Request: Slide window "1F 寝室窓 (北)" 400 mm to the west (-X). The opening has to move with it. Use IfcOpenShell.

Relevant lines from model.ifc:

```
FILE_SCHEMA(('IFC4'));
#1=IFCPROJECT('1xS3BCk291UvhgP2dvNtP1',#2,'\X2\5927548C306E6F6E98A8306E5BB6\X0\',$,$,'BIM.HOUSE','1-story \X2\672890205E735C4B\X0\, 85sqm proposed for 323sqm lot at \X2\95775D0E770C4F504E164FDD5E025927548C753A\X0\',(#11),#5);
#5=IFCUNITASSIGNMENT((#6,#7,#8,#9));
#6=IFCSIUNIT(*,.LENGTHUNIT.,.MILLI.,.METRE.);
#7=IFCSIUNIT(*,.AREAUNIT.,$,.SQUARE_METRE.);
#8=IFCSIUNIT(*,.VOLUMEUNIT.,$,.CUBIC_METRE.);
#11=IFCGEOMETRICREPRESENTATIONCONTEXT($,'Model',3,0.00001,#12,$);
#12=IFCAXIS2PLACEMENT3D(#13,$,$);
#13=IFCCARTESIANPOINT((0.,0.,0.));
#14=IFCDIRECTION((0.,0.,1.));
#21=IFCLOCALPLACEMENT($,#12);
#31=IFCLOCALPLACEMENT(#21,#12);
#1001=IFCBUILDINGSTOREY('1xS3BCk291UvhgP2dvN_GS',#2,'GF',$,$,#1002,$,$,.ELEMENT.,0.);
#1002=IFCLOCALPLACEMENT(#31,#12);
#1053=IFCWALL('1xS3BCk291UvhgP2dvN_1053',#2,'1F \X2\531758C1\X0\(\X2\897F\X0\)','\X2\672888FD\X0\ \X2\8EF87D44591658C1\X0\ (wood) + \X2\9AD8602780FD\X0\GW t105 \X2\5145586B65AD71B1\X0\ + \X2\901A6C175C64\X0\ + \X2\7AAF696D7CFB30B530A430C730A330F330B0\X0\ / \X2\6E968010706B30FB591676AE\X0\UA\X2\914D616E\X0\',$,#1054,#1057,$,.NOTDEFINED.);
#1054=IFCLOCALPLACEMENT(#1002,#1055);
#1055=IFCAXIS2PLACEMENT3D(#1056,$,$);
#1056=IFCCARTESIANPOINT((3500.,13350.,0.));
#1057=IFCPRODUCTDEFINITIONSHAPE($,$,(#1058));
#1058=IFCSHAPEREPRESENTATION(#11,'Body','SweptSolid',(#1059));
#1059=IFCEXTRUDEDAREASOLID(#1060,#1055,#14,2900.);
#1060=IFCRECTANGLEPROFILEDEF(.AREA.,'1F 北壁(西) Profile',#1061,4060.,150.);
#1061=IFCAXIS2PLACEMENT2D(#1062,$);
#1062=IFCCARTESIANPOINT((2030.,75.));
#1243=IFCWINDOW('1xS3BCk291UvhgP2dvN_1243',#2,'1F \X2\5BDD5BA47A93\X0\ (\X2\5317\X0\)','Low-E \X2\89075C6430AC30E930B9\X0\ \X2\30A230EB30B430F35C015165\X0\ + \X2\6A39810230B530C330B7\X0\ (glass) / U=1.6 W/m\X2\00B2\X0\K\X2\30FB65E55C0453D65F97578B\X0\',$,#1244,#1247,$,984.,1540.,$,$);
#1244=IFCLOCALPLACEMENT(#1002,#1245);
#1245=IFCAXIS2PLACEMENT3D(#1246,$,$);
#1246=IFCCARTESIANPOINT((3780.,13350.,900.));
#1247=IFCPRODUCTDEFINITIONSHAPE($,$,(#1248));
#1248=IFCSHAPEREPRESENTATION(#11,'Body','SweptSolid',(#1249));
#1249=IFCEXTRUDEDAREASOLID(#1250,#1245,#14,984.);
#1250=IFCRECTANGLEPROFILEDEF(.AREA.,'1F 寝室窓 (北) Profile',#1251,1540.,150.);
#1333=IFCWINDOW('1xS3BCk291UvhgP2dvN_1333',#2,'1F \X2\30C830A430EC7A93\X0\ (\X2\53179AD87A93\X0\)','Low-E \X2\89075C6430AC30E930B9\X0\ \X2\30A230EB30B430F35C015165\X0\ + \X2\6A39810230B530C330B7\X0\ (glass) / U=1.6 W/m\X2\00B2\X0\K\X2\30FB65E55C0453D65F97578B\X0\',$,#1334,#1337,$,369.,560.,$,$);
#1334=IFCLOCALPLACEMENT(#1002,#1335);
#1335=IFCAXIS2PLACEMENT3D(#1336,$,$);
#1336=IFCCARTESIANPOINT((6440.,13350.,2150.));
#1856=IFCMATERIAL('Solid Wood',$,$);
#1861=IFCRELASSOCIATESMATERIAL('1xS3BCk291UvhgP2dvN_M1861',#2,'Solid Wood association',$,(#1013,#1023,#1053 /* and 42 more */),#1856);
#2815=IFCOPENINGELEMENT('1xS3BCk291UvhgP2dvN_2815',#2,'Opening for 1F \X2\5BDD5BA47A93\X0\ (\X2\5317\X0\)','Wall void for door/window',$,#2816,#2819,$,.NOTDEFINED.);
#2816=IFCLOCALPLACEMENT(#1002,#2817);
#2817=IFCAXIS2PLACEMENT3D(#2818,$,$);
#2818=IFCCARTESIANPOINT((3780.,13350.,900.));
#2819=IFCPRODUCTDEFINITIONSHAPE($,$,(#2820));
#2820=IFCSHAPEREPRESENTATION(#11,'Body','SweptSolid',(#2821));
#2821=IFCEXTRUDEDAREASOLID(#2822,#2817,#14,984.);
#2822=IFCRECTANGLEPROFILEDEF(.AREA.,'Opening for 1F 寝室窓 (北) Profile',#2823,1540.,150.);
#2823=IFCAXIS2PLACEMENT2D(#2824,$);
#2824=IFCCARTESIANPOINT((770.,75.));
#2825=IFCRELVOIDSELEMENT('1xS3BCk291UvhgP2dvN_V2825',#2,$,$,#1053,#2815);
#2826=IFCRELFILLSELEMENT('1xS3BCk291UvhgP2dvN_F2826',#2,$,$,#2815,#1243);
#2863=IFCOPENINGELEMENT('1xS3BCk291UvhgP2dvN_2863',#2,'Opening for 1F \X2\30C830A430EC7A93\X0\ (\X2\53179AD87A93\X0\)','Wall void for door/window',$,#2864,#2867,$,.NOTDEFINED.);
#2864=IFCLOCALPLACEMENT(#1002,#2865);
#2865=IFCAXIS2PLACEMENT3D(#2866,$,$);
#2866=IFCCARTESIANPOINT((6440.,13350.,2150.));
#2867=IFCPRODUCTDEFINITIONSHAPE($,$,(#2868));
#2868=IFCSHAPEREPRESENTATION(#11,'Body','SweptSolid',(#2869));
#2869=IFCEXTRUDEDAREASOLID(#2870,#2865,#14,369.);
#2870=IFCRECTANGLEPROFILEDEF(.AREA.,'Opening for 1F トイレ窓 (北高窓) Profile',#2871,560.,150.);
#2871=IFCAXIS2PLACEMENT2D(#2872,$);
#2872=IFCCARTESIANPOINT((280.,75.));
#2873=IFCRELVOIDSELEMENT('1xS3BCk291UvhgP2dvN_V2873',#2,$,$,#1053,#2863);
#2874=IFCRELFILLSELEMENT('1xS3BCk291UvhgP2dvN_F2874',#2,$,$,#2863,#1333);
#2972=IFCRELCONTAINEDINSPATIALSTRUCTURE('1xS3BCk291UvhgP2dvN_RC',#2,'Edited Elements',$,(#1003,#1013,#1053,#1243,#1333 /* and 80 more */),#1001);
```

```python
import ifcopenshell
import ifcopenshell.api.geometry
import ifcopenshell.util.placement

model = ifcopenshell.open("model.ifc")

window = model.by_guid("1xS3BCk291UvhgP2dvN_1243")
opening = window.FillsVoids[0].RelatingOpeningElement
wall = opening.VoidsElements[0].RelatingBuildingElement

wall_matrix = ifcopenshell.util.placement.get_local_placement(wall.ObjectPlacement)
shift = wall_matrix[:3, 0] * -400.0
before = ifcopenshell.util.placement.get_local_placement(window.ObjectPlacement)[:3, 3].copy()

# The window is not placed relative to its opening, so move both.
for product in (opening, window):
    matrix = ifcopenshell.util.placement.get_local_placement(product.ObjectPlacement)
    matrix[:3, 3] += shift
    ifcopenshell.api.geometry.edit_object_placement(model, product=product, matrix=matrix, is_si=False)

after = ifcopenshell.util.placement.get_local_placement(window.ObjectPlacement)[:3, 3]
print("window moved by", (after - before).round(3) + 0.0)

model.write("model_updated.ifc")
```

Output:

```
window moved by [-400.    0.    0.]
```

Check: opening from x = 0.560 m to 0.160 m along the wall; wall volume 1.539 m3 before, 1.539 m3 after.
